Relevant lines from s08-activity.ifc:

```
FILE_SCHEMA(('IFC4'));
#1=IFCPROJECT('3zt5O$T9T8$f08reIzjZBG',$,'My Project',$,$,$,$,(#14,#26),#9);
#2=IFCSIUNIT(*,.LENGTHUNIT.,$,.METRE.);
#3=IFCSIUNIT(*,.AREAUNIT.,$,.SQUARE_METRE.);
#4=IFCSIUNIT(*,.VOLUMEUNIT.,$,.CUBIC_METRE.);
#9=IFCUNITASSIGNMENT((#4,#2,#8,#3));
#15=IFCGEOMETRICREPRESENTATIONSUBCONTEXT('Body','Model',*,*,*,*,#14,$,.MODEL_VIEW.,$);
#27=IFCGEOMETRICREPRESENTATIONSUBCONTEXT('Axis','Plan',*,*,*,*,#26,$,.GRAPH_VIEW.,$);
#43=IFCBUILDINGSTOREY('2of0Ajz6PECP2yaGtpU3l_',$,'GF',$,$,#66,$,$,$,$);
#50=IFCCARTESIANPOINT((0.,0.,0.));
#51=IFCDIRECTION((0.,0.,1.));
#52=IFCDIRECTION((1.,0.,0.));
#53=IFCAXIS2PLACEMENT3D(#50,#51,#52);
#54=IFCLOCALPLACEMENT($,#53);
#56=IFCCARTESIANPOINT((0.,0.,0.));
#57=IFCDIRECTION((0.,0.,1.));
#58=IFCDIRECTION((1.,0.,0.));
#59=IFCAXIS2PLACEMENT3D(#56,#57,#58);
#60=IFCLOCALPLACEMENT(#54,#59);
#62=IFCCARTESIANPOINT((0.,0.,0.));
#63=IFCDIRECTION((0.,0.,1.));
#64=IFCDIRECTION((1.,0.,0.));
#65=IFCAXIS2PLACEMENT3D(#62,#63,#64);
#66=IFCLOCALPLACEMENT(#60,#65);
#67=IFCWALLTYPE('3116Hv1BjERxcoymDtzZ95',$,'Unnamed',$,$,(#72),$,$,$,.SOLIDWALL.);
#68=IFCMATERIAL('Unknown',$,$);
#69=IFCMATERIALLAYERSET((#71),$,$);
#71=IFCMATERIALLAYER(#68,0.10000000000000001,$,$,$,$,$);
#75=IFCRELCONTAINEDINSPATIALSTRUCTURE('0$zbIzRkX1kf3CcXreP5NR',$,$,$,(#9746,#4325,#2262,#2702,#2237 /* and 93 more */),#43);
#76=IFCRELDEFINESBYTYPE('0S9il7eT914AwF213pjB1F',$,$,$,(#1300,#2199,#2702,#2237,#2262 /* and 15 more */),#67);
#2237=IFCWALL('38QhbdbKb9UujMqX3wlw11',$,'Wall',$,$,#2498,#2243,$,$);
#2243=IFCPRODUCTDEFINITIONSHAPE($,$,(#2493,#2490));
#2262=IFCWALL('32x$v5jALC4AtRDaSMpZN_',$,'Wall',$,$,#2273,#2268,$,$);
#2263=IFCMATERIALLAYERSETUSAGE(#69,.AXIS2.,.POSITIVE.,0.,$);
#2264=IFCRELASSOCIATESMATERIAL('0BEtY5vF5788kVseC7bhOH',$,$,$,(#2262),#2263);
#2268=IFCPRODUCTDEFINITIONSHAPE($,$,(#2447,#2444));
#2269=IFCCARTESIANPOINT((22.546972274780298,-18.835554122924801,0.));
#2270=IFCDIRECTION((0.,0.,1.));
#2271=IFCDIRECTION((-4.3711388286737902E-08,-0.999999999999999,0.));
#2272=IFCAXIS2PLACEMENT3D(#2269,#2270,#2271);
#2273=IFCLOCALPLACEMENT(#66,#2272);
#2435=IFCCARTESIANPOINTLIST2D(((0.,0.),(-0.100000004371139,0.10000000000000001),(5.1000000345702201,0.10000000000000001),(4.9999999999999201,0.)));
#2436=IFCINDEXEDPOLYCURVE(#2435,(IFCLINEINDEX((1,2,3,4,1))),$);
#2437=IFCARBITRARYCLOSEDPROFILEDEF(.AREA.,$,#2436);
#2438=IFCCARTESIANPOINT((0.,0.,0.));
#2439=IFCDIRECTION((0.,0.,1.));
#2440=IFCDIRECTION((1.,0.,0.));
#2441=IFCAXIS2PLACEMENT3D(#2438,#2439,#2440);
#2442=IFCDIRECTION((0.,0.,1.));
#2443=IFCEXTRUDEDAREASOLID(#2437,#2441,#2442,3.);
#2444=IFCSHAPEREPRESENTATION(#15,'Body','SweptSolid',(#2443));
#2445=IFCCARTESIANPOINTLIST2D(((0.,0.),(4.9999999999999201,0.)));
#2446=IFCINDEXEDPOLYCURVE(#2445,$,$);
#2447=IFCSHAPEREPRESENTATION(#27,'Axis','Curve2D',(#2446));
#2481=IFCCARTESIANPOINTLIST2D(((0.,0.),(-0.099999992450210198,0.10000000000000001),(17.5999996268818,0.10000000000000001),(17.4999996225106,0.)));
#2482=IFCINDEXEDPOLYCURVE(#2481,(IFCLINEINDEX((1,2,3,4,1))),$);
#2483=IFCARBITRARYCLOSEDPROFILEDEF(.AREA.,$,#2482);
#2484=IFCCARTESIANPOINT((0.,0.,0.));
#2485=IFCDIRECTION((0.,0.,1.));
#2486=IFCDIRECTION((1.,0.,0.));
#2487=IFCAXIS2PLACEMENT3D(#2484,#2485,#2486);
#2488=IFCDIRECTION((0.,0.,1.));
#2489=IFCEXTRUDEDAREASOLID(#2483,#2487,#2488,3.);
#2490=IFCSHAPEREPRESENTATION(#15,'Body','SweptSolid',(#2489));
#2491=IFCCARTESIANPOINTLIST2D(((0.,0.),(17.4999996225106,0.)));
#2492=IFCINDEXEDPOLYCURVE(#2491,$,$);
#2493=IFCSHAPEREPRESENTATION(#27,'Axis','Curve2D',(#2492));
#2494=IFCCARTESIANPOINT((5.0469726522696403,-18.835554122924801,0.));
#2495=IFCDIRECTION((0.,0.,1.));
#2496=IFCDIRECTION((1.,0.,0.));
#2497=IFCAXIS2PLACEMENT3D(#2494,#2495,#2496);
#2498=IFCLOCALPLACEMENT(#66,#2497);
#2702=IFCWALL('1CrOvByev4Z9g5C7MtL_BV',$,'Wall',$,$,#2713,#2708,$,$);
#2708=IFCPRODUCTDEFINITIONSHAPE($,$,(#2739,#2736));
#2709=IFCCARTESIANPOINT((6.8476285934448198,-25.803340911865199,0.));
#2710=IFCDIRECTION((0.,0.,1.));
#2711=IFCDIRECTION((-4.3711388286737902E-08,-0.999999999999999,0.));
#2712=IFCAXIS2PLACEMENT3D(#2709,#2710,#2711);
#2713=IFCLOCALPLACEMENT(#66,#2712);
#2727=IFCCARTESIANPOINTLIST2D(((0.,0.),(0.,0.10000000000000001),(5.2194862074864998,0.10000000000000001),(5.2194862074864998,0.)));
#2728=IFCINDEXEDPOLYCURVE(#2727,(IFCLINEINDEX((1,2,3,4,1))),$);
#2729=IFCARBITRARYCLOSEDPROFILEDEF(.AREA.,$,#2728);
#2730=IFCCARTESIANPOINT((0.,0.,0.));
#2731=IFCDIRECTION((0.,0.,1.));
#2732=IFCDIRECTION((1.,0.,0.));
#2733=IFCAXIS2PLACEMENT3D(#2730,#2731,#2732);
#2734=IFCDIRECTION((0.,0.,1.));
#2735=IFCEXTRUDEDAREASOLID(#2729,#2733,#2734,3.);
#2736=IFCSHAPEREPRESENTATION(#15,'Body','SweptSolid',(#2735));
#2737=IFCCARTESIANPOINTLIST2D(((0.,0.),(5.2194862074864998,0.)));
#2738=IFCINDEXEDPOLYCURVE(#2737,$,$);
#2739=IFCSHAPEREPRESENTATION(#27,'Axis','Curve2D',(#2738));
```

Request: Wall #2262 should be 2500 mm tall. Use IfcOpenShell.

```python
import ifcopenshell
import ifcopenshell.geom
import ifcopenshell.util.representation
import ifcopenshell.util.shape
import ifcopenshell.util.unit

model = ifcopenshell.open("s08-activity.ifc")
unit_scale = ifcopenshell.util.unit.calculate_unit_scale(model)
settings = ifcopenshell.geom.settings()


def volume(element):
    """Net volume in cubic metres, openings subtracted."""
    shape = ifcopenshell.geom.create_shape(settings, element)
    return ifcopenshell.util.shape.get_volume(shape.geometry)


wall = model.by_guid("32x$v5jALC4AtRDaSMpZN_")
before = volume(wall)

body = ifcopenshell.util.representation.get_representation(wall, "Model", "Body")
solid = body.Items[0]
old_height = solid.Depth
solid.Depth = 2.5 / unit_scale
after = volume(wall)

print(f"height {old_height:g} -> {solid.Depth:g}, volume {before:.3f} -> {after:.3f} m3")

model.write("s08-activity_updated.ifc")
```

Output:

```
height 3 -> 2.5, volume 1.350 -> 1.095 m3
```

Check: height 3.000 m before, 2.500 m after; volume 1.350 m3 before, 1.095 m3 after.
